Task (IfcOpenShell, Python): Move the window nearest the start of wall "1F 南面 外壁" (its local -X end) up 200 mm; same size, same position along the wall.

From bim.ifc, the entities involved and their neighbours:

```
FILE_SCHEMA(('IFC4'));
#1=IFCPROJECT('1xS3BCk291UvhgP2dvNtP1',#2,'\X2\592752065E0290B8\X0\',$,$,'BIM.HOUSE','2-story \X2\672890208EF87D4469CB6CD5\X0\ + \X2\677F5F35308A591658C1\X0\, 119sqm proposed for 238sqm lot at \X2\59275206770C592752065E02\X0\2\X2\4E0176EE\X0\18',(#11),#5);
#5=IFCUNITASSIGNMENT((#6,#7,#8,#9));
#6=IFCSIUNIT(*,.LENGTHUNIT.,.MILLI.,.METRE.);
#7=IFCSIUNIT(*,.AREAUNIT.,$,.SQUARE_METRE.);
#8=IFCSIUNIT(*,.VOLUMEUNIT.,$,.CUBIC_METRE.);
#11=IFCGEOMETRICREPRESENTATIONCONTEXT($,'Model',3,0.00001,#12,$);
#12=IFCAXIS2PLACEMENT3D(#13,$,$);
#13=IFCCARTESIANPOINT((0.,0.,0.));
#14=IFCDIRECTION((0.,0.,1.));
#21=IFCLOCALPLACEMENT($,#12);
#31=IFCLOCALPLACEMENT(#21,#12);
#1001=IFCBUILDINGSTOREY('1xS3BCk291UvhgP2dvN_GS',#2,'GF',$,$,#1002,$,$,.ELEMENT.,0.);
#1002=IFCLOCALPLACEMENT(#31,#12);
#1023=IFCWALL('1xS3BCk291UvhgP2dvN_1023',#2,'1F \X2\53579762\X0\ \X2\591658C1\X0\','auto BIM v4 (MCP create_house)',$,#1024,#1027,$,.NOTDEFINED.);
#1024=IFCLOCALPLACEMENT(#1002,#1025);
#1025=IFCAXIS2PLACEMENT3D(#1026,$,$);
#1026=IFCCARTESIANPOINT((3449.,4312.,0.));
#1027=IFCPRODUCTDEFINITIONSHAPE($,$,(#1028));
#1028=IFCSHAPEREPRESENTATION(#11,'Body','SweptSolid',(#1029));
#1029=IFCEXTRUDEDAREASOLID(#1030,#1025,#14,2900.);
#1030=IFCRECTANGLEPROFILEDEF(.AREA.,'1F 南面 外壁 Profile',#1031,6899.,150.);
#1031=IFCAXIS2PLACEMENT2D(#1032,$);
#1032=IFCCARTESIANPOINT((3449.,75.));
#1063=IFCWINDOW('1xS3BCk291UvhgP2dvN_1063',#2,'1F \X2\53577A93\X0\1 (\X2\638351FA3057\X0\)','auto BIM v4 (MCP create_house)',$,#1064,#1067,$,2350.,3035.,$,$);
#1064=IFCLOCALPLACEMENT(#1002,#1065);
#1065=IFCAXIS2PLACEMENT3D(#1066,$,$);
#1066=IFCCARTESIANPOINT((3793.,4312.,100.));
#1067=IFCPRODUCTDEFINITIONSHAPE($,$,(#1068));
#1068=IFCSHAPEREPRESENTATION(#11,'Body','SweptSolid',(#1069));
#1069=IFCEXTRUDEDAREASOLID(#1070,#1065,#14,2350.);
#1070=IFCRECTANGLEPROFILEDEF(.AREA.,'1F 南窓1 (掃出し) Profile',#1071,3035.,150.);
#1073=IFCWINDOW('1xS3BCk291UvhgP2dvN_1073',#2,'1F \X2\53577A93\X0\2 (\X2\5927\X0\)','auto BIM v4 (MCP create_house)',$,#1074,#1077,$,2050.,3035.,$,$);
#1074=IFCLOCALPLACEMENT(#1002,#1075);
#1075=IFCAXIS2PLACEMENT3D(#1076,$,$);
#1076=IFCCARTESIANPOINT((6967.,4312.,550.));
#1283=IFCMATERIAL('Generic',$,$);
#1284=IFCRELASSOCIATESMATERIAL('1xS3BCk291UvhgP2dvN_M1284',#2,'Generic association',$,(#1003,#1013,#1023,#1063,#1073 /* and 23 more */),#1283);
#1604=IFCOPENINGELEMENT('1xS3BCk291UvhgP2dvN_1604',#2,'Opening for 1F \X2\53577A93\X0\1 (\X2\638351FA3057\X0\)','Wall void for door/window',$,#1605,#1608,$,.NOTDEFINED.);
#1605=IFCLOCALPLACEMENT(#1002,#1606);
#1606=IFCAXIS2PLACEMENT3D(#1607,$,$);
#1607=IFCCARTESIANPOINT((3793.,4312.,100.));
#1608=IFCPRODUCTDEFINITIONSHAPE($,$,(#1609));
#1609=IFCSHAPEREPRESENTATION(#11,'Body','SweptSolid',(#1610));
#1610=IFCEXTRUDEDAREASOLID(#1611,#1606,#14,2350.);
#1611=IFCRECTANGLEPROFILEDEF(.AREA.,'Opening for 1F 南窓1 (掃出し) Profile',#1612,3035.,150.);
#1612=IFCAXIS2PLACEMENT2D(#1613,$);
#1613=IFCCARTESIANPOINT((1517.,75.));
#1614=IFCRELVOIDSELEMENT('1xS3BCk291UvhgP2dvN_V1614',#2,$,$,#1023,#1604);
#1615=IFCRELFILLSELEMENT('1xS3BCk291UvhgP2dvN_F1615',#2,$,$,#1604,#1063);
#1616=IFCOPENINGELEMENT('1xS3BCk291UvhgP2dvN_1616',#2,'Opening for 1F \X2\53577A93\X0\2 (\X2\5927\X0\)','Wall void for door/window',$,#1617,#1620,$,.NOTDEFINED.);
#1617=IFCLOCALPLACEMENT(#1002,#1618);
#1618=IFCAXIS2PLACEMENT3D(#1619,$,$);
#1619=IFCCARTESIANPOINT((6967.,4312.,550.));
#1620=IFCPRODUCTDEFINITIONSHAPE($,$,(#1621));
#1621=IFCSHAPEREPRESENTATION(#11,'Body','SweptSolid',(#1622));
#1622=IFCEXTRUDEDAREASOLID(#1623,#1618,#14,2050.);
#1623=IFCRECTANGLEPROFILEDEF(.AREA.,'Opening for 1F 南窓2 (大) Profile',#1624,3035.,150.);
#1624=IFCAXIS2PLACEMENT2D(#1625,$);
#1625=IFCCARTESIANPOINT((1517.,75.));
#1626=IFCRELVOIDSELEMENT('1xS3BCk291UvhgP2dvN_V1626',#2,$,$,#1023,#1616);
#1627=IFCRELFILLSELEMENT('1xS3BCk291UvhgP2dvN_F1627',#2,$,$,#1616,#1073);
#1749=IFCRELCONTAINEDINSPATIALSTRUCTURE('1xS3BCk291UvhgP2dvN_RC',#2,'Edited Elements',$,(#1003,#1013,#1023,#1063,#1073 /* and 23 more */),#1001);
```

```python
import numpy as np
import ifcopenshell
import ifcopenshell.api.geometry
import ifcopenshell.util.placement
import ifcopenshell.util.unit

model = ifcopenshell.open("bim.ifc")
unit_scale = ifcopenshell.util.unit.calculate_unit_scale(model)

window = model.by_guid("1xS3BCk291UvhgP2dvN_1063")
opening = window.FillsVoids[0].RelatingOpeningElement
dz = 0.2 / unit_scale

shift = np.array([0.0, 0.0, dz])
# The window is not placed relative to its opening, so move both.
for product in (opening, window):
    matrix = ifcopenshell.util.placement.get_local_placement(product.ObjectPlacement)
    matrix[:3, 3] += shift
    ifcopenshell.api.geometry.edit_object_placement(model, product=product, matrix=matrix, is_si=False)

print(f"moved by {dz * unit_scale:+.3f} m")

model.write("bim_rev.ifc")
```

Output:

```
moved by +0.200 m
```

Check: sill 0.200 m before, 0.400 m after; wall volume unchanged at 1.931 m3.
